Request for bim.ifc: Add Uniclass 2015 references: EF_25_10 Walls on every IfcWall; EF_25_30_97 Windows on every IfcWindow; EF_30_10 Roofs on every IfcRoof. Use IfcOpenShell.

First a look at what the model holds.

```python
import ifcopenshell

model = ifcopenshell.open("bim.ifc")
print(model.schema)
print("classifications:", [c.Name for c in model.by_type("IfcClassification")])
for ifc_class in ("IfcDoor", "IfcRoof", "IfcStair", "IfcWall", "IfcWindow"):
    print(ifc_class, len(model.by_type(ifc_class)))
```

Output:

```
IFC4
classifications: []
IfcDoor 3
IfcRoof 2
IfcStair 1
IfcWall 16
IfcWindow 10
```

```python
import ifcopenshell
import ifcopenshell.api.classification

model = ifcopenshell.open("bim.ifc")

system = ifcopenshell.api.classification.add_classification(model, classification="Uniclass 2015")

codes = {
    "IfcWall": ("EF_25_10", "Walls"),
    "IfcWindow": ("EF_25_30_97", "Windows"),
    "IfcRoof": ("EF_30_10", "Roofs"),
}
for ifc_class, (code, name) in codes.items():
    products = model.by_type(ifc_class)
    ifcopenshell.api.classification.add_reference(
        model, products=products, classification=system, identification=code, name=name
    )
    print(code, len(products))

model.write("bim_rev.ifc")
```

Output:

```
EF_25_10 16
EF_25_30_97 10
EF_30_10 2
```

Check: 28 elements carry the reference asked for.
